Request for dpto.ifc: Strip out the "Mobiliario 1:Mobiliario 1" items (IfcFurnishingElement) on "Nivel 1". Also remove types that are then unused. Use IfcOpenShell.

First a look at what the model holds.

```python
import ifcopenshell
import ifcopenshell.util.element

model = ifcopenshell.open("dpto.ifc")
print(model.schema)
storey = next(s for s in model.by_type("IfcBuildingStorey") if s.Name == "Nivel 1")
furniture = [e for e in ifcopenshell.util.element.get_decomposition(storey) if e.is_a("IfcFurnishingElement")]
seen = {}
for e in furniture:
    element_type = ifcopenshell.util.element.get_type(e)
    name = element_type.Name if element_type not in (None, e) else None
    seen[name] = seen.get(name, 0) + 1
for name, count in sorted(seen.items(), key=str):
    print(count, "x", name)
```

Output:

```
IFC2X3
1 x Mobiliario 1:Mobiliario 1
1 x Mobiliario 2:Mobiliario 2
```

```python
import ifcopenshell
import ifcopenshell.api.root
import ifcopenshell.util.element

model = ifcopenshell.open("dpto.ifc")

storey = next(s for s in model.by_type("IfcBuildingStorey") if s.Name == "Nivel 1")
furniture = [e for e in ifcopenshell.util.element.get_decomposition(storey) if e.is_a("IfcFurnishingElement")]
targets = [e for e in furniture if (t := ifcopenshell.util.element.get_type(e)) not in (None, e) and t.Name == "Mobiliario 1:Mobiliario 1"]
types = {ifcopenshell.util.element.get_type(e) for e in targets} - {None, *targets}

for e in targets:
    ifcopenshell.api.root.remove_product(model, product=e)
print(len(targets), "removed")

unused = [t for t in types if not ifcopenshell.util.element.get_types(t)]
for t in unused:
    ifcopenshell.api.root.remove_product(model, product=t)
print(len(unused), "unused types removed")

model.write("dpto_rev.ifc")
```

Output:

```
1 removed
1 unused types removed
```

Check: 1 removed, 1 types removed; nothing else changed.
